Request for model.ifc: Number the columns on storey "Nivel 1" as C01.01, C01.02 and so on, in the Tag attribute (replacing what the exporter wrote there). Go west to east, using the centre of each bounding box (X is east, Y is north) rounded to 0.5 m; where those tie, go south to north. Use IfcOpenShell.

First a look at what the model holds.

```python
import ifcopenshell
import ifcopenshell.util.element
import ifcopenshell.util.placement

model = ifcopenshell.open("model.ifc")
print(model.schema)
storey = next(s for s in model.by_type("IfcBuildingStorey") if s.Name == "Nivel 1")
columns = [e for e in ifcopenshell.util.element.get_decomposition(storey) if e.is_a("IfcColumn")]
for e in sorted(columns, key=lambda e: e.id()):
    origin = ifcopenshell.util.placement.get_local_placement(e.ObjectPlacement)[:3, 3]
    print(e.id(), e.Tag, e.Name, origin.round(2) + 0.0, sep=" | ")
```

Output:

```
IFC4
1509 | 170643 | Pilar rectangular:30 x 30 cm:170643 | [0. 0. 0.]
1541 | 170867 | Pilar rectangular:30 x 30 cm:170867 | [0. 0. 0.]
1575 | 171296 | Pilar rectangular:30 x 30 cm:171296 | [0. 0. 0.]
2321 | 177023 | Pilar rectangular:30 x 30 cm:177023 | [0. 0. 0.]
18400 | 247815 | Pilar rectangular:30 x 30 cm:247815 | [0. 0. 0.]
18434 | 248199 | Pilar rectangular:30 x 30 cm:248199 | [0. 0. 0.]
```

```python
import ifcopenshell
import ifcopenshell.geom
import ifcopenshell.util.element
import ifcopenshell.util.shape

model = ifcopenshell.open("model.ifc")
settings = ifcopenshell.geom.settings()
settings.set("use-world-coords", True)


def centre(element):
    shape = ifcopenshell.geom.create_shape(settings, element)
    return ifcopenshell.util.shape.get_bbox_centroid(shape.geometry)


storey = next(s for s in model.by_type("IfcBuildingStorey") if s.Name == "Nivel 1")
columns = [e for e in ifcopenshell.util.element.get_decomposition(storey) if e.is_a("IfcColumn")]

# Insertion points can sit at a corner or the storey origin, so sort by the geometry (in metres).
centres = {e: centre(e) for e in columns}
columns.sort(key=lambda e: (round(centres[e][0] / 0.5), centres[e][1]))

for i, e in enumerate(columns, start=1):
    number = f"C01.{i:02d}"
    e.Tag = number
    print(e.id(), number)

model.write("model_edited.ifc")
```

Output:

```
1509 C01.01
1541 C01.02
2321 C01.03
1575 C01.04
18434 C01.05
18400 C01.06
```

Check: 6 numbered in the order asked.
